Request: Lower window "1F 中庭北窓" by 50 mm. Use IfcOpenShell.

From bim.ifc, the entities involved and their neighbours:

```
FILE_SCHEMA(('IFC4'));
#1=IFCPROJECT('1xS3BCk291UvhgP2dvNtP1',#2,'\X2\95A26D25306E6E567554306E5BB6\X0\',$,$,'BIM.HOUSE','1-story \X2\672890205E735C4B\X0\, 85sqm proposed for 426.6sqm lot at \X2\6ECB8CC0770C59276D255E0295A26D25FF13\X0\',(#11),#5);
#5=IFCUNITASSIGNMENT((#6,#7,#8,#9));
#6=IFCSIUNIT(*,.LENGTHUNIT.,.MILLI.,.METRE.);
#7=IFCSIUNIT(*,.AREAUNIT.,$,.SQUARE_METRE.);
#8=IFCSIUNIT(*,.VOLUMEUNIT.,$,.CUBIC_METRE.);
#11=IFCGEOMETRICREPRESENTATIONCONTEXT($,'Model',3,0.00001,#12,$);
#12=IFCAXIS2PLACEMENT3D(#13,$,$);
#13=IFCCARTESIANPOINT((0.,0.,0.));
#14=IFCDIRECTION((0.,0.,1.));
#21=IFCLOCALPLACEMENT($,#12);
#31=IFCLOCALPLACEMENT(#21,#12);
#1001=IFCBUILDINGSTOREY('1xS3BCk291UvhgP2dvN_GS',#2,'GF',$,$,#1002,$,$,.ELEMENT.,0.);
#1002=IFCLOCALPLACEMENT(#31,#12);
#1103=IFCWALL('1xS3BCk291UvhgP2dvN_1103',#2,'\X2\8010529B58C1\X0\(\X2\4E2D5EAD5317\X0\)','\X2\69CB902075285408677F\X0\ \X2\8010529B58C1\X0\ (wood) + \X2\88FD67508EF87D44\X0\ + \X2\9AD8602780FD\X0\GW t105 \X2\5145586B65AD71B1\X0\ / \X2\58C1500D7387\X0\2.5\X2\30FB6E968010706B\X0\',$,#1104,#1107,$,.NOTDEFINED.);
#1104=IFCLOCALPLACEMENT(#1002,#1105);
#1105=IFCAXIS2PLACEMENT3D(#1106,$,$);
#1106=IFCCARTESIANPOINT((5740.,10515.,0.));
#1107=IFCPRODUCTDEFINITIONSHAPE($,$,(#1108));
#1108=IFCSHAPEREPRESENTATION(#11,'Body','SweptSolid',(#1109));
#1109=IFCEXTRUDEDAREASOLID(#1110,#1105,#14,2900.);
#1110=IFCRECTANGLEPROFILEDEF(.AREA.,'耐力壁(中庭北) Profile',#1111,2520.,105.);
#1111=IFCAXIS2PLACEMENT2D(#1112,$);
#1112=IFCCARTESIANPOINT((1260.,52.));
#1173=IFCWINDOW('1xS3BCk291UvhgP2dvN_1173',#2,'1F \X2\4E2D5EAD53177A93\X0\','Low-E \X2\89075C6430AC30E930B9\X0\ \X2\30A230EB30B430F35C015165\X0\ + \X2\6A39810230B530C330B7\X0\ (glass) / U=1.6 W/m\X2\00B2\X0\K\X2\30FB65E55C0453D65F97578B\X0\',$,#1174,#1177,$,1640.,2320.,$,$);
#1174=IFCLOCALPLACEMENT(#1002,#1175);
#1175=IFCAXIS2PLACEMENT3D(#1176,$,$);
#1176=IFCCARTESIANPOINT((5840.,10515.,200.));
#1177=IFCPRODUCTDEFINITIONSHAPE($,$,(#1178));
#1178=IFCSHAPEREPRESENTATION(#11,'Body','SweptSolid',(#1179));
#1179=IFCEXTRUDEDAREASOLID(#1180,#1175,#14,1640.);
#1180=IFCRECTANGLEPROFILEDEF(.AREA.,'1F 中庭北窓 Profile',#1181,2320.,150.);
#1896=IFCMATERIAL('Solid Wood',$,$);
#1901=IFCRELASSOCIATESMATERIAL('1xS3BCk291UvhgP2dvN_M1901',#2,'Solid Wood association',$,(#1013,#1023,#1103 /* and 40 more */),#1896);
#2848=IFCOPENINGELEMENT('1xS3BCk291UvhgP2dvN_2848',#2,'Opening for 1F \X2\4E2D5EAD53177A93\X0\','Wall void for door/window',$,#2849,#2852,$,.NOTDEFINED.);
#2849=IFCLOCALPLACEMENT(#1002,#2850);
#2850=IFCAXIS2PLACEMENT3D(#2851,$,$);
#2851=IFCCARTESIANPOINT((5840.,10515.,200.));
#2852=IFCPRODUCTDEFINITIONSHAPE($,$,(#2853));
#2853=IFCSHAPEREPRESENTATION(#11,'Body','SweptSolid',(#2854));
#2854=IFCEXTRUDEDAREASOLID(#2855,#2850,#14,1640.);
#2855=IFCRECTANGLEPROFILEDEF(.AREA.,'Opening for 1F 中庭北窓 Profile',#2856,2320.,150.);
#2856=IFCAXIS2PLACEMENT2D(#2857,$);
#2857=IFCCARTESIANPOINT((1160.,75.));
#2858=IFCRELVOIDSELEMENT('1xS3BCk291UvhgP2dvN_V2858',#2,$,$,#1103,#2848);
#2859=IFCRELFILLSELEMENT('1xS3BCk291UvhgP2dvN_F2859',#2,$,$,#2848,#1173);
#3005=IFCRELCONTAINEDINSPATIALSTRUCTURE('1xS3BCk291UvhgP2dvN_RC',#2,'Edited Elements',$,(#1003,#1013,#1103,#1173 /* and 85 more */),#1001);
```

```python
import numpy as np
import ifcopenshell
import ifcopenshell.api.geometry
import ifcopenshell.util.placement
import ifcopenshell.util.unit

model = ifcopenshell.open("bim.ifc")
unit_scale = ifcopenshell.util.unit.calculate_unit_scale(model)

window = model.by_guid("1xS3BCk291UvhgP2dvN_1173")
opening = window.FillsVoids[0].RelatingOpeningElement
dz = -0.05 / unit_scale

shift = np.array([0.0, 0.0, dz])
# The window is not placed relative to its opening, so move both.
for product in (opening, window):
    matrix = ifcopenshell.util.placement.get_local_placement(product.ObjectPlacement)
    matrix[:3, 3] += shift
    ifcopenshell.api.geometry.edit_object_placement(model, product=product, matrix=matrix, is_si=False)

print(f"moved by {dz * unit_scale:+.3f} m")

model.write("bim_rev.ifc")
```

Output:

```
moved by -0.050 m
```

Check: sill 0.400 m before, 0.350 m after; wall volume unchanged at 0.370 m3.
